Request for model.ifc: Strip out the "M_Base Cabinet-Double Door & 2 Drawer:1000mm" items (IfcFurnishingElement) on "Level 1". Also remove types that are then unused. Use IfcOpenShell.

First a look at what the model holds.

```python
import ifcopenshell
import ifcopenshell.util.element

model = ifcopenshell.open("model.ifc")
print(model.schema)
storey = next(s for s in model.by_type("IfcBuildingStorey") if s.Name == "Level 1")
furniture = [e for e in ifcopenshell.util.element.get_decomposition(storey) if e.is_a("IfcFurnishingElement")]
seen = {}
for e in furniture:
    element_type = ifcopenshell.util.element.get_type(e)
    name = element_type.Name if element_type not in (None, e) else None
    seen[name] = seen.get(name, 0) + 1
for name, count in sorted(seen.items(), key=str):
    print(count, "x", name)
```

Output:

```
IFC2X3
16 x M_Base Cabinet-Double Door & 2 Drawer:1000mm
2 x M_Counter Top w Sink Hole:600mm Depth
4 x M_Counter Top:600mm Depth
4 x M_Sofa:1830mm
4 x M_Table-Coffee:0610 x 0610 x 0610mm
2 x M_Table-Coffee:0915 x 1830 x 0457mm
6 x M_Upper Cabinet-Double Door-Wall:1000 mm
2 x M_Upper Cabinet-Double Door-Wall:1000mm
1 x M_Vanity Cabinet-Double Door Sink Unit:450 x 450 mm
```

```python
import ifcopenshell
import ifcopenshell.api.root
import ifcopenshell.util.element

model = ifcopenshell.open("model.ifc")

storey = next(s for s in model.by_type("IfcBuildingStorey") if s.Name == "Level 1")
furniture = [e for e in ifcopenshell.util.element.get_decomposition(storey) if e.is_a("IfcFurnishingElement")]
targets = [e for e in furniture if (t := ifcopenshell.util.element.get_type(e)) not in (None, e) and t.Name == "M_Base Cabinet-Double Door & 2 Drawer:1000mm"]
types = {ifcopenshell.util.element.get_type(e) for e in targets} - {None, *targets}

for e in targets:
    ifcopenshell.api.root.remove_product(model, product=e)
print(len(targets), "removed")

unused = [t for t in types if not ifcopenshell.util.element.get_types(t)]
for t in unused:
    ifcopenshell.api.root.remove_product(model, product=t)
print(len(unused), "unused types removed")

model.write("model_updated.ifc")
```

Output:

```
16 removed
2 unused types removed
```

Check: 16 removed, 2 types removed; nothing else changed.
